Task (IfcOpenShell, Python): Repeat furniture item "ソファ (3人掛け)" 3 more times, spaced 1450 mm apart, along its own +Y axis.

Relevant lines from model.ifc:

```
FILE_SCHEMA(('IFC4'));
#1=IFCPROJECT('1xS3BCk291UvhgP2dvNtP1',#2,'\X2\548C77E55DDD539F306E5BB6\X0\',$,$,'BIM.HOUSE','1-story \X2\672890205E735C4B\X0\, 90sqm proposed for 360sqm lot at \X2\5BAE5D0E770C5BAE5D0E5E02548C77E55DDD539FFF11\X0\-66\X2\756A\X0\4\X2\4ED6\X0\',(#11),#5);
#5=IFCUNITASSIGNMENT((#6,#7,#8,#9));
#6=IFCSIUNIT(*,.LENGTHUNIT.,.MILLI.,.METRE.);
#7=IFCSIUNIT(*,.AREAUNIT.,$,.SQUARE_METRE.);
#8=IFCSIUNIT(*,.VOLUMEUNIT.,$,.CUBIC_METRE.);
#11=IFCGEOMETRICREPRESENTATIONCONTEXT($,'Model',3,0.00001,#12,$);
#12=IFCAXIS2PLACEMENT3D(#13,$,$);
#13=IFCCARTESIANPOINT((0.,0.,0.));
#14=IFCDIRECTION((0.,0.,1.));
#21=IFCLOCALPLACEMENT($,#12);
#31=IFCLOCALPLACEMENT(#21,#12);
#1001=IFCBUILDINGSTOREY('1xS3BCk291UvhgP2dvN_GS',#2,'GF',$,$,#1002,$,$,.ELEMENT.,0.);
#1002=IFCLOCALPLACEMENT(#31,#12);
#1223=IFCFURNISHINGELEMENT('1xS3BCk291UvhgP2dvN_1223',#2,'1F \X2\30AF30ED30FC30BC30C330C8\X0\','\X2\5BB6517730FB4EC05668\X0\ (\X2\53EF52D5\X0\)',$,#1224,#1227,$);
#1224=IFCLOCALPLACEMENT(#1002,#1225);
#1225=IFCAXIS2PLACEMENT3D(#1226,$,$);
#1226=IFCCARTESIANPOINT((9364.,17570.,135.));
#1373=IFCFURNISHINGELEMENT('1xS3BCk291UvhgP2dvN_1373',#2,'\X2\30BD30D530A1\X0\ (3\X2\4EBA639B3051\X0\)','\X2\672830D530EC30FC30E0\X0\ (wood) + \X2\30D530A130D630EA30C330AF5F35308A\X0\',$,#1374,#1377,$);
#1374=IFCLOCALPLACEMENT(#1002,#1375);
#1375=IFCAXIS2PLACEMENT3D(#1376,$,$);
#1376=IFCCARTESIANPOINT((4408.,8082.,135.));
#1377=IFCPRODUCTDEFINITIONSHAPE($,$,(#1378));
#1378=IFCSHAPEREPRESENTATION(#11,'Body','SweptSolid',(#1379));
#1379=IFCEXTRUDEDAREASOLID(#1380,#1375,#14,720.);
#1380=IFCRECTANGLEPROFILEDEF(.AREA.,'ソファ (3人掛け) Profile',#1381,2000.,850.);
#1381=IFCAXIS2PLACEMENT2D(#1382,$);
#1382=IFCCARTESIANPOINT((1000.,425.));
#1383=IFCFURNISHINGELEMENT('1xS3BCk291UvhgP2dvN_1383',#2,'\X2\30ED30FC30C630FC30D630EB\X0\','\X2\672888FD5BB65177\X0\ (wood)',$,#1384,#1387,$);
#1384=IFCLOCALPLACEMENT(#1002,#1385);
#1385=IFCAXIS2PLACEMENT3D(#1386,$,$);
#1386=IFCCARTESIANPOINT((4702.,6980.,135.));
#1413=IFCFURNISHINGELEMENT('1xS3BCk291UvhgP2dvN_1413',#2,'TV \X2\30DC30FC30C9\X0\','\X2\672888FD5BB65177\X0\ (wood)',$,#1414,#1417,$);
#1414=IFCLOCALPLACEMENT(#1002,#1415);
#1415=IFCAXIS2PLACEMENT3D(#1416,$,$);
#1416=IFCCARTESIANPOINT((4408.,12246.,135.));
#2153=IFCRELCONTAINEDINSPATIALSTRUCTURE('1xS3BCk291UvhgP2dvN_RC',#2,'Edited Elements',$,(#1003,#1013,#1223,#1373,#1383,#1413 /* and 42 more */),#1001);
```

```python
import ifcopenshell
import ifcopenshell.api.geometry
import ifcopenshell.api.root
import ifcopenshell.util.element
import ifcopenshell.util.placement
import ifcopenshell.util.unit

model = ifcopenshell.open("model.ifc")
unit_scale = ifcopenshell.util.unit.calculate_unit_scale(model)


def reuse_history(source, copy):
    """copy_class also copies each property set's owner history, people and application; keep the originals."""
    for rel in copy.IsDefinedBy:
        if rel.is_a("IfcRelDefinesByProperties") and (history := rel.RelatingPropertyDefinition.OwnerHistory):
            rel.RelatingPropertyDefinition.OwnerHistory = source.OwnerHistory
            ifcopenshell.util.element.remove_deep2(model, history)


source = model.by_guid("1xS3BCk291UvhgP2dvN_1373")
base = ifcopenshell.util.placement.get_local_placement(source.ObjectPlacement)
step = base[:3, 1] * 1.45 / unit_scale

for i in range(1, 4):
    copy = ifcopenshell.api.root.copy_class(model, product=source)
    copy.Representation = ifcopenshell.util.element.copy_deep(
        model, source.Representation, exclude=["IfcGeometricRepresentationContext", "IfcRepresentationMap"]
    )
    reuse_history(source, copy)
    matrix = base.copy()
    matrix[:3, 3] += i * step
    print("added at", matrix[:3, 3].round(3) + 0.0)
    ifcopenshell.api.geometry.edit_object_placement(model, product=copy, matrix=matrix, is_si=False)

model.write("model_rev.ifc")
```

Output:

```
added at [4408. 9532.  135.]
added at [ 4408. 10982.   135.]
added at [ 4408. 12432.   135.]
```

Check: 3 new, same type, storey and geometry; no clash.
